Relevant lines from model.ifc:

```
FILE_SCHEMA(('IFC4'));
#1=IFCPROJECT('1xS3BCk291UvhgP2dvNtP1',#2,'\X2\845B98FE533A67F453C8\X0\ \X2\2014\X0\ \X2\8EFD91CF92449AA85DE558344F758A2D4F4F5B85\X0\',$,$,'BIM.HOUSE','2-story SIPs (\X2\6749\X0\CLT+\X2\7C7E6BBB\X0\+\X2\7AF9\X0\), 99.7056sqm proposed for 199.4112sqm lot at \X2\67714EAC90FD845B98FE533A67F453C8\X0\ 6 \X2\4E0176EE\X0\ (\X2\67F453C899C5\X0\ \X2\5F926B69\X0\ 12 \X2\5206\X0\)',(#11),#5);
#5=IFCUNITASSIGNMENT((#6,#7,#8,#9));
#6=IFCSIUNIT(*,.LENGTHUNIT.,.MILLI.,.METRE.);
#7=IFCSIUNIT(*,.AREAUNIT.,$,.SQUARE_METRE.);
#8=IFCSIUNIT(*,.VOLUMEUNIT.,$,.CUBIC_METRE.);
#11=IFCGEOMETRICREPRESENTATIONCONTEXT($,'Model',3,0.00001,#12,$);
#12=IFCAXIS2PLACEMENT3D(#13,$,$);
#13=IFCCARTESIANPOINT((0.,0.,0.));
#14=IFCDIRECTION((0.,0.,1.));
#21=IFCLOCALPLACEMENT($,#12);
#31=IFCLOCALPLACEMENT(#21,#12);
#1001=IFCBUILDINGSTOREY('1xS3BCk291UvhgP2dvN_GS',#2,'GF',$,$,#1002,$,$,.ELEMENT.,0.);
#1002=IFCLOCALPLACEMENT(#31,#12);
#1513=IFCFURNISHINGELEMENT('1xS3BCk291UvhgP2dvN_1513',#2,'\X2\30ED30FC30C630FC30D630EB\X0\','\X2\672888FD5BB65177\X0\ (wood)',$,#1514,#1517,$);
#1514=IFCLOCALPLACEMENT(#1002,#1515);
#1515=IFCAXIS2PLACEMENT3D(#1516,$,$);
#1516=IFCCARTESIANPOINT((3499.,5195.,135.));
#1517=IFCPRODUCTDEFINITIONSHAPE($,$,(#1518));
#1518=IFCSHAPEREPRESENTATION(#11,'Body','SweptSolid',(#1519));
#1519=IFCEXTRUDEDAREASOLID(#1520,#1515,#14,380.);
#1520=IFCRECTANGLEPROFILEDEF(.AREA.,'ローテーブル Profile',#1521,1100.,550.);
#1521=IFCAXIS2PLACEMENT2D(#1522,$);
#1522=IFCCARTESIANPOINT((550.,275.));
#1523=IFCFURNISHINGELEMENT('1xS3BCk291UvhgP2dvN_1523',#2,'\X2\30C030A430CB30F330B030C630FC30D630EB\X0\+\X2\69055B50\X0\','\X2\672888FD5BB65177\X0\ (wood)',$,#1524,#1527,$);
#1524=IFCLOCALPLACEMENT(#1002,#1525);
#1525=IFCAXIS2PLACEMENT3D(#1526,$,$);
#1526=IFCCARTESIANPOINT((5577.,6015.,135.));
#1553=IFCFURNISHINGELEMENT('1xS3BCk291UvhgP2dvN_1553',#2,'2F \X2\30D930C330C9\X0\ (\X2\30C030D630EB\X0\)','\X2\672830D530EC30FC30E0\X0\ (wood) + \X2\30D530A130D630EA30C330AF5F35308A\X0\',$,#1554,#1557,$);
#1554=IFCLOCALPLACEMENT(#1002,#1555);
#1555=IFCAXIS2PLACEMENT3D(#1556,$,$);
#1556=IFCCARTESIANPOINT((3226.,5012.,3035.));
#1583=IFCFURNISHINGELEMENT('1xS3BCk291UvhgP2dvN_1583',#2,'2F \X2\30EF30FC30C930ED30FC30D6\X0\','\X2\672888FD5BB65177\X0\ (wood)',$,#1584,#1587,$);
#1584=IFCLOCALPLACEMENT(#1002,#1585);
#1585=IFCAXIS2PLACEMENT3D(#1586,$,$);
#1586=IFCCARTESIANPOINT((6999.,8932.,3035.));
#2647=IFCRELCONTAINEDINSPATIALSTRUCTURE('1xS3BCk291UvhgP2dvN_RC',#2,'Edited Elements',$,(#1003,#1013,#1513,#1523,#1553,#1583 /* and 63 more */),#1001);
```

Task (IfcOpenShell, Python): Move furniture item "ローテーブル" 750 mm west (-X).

```python
import ifcopenshell
import ifcopenshell.api.geometry
import ifcopenshell.util.placement

model = ifcopenshell.open("model.ifc")

item = model.by_id(1513)
matrix = ifcopenshell.util.placement.get_local_placement(item.ObjectPlacement)
matrix[0, 3] -= 750.0
ifcopenshell.api.geometry.edit_object_placement(model, product=item, matrix=matrix, is_si=False)

print(ifcopenshell.util.placement.get_local_placement(item.ObjectPlacement).round(3) + 0.0)

model.write("model_v2.ifc")
```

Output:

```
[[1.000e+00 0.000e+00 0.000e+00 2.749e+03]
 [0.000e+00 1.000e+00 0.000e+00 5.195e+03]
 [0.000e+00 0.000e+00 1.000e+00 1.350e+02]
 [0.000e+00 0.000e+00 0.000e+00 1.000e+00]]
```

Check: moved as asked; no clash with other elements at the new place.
